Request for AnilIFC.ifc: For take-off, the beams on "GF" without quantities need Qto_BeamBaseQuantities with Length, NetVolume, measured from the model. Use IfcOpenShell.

First a look at what the model holds.

```python
import ifcopenshell
import ifcopenshell.util.element
import ifcopenshell.util.unit

model = ifcopenshell.open("AnilIFC.ifc")
print(model.schema)
for unit_type in ("LENGTHUNIT", "AREAUNIT", "VOLUMEUNIT"):
    print(unit_type, ifcopenshell.util.unit.calculate_unit_scale(model, unit_type))
storey = next(s for s in model.by_type("IfcBuildingStorey") if s.Name == "GF")
beams = [e for e in ifcopenshell.util.element.get_decomposition(storey) if e.is_a("IfcBeam")]
for e in sorted(beams, key=lambda e: e.id()):
    print(e.id(), e.is_a(), e.Name, list(ifcopenshell.util.element.get_psets(e, qtos_only=True)), sep=" | ")
```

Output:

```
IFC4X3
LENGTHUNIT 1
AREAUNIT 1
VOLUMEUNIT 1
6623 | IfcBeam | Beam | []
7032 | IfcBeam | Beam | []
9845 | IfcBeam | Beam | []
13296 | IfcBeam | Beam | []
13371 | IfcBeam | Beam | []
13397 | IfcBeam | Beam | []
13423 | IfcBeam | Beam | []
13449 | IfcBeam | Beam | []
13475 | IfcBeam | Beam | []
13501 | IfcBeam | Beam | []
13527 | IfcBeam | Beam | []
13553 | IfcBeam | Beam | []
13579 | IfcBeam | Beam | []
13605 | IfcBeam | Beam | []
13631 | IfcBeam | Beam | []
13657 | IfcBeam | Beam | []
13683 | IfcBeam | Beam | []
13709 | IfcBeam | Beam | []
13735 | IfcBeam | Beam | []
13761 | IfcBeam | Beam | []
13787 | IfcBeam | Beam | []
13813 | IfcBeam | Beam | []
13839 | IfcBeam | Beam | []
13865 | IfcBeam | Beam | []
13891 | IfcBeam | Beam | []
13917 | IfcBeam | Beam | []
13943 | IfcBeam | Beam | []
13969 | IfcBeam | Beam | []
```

```python
import ifcopenshell
import ifcopenshell.api.pset
import ifcopenshell.geom
import ifcopenshell.util.element
import ifcopenshell.util.shape
import ifcopenshell.util.unit

model = ifcopenshell.open("AnilIFC.ifc")
unit_scale = ifcopenshell.util.unit.calculate_unit_scale(model)
volume_scale = ifcopenshell.util.unit.calculate_unit_scale(model, "VOLUMEUNIT")
settings = ifcopenshell.geom.settings()

storey = next(s for s in model.by_type("IfcBuildingStorey") if s.Name == "GF")
beams = [e for e in ifcopenshell.util.element.get_decomposition(storey) if e.is_a("IfcBeam")]

for e in sorted(beams, key=lambda e: e.id()):
    if ifcopenshell.util.element.get_psets(e, qtos_only=True, should_inherit=False):
        continue
    # Geometry comes back in metres, in the element's own axes.
    shape = ifcopenshell.geom.create_shape(settings, e)
    values = {
        "Length": ifcopenshell.util.shape.get_max_xyz(shape.geometry) / unit_scale,
        "NetVolume": ifcopenshell.util.shape.get_volume(shape.geometry) / volume_scale,
    }
    qto = ifcopenshell.api.pset.add_qto(model, product=e, name="Qto_BeamBaseQuantities")
    ifcopenshell.api.pset.edit_qto(model, qto=qto, properties=values)
    print(e.id(), {k: round(v, 3) for k, v in values.items()})

model.write("AnilIFC-out.ifc")
```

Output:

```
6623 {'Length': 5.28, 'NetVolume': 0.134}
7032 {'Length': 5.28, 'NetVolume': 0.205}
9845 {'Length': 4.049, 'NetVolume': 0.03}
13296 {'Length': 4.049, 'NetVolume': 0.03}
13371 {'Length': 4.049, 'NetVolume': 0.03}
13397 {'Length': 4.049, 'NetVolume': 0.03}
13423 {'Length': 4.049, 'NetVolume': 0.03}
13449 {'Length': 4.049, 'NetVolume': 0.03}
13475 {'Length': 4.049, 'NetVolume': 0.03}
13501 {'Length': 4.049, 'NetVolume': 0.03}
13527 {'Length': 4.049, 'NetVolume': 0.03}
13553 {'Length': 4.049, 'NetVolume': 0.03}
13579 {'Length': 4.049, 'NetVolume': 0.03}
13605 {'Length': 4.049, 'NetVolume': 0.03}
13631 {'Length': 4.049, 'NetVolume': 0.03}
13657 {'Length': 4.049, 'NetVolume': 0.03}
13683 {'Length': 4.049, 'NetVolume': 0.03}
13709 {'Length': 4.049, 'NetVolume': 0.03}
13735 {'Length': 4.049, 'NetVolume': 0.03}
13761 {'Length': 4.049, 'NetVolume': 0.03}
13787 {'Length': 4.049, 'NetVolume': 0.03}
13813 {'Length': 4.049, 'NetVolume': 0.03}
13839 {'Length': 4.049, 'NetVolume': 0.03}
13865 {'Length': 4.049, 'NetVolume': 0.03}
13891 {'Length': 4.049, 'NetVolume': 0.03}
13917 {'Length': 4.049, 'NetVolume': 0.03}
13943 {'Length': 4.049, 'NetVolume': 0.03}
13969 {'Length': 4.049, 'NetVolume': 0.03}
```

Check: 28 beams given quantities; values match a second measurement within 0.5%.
